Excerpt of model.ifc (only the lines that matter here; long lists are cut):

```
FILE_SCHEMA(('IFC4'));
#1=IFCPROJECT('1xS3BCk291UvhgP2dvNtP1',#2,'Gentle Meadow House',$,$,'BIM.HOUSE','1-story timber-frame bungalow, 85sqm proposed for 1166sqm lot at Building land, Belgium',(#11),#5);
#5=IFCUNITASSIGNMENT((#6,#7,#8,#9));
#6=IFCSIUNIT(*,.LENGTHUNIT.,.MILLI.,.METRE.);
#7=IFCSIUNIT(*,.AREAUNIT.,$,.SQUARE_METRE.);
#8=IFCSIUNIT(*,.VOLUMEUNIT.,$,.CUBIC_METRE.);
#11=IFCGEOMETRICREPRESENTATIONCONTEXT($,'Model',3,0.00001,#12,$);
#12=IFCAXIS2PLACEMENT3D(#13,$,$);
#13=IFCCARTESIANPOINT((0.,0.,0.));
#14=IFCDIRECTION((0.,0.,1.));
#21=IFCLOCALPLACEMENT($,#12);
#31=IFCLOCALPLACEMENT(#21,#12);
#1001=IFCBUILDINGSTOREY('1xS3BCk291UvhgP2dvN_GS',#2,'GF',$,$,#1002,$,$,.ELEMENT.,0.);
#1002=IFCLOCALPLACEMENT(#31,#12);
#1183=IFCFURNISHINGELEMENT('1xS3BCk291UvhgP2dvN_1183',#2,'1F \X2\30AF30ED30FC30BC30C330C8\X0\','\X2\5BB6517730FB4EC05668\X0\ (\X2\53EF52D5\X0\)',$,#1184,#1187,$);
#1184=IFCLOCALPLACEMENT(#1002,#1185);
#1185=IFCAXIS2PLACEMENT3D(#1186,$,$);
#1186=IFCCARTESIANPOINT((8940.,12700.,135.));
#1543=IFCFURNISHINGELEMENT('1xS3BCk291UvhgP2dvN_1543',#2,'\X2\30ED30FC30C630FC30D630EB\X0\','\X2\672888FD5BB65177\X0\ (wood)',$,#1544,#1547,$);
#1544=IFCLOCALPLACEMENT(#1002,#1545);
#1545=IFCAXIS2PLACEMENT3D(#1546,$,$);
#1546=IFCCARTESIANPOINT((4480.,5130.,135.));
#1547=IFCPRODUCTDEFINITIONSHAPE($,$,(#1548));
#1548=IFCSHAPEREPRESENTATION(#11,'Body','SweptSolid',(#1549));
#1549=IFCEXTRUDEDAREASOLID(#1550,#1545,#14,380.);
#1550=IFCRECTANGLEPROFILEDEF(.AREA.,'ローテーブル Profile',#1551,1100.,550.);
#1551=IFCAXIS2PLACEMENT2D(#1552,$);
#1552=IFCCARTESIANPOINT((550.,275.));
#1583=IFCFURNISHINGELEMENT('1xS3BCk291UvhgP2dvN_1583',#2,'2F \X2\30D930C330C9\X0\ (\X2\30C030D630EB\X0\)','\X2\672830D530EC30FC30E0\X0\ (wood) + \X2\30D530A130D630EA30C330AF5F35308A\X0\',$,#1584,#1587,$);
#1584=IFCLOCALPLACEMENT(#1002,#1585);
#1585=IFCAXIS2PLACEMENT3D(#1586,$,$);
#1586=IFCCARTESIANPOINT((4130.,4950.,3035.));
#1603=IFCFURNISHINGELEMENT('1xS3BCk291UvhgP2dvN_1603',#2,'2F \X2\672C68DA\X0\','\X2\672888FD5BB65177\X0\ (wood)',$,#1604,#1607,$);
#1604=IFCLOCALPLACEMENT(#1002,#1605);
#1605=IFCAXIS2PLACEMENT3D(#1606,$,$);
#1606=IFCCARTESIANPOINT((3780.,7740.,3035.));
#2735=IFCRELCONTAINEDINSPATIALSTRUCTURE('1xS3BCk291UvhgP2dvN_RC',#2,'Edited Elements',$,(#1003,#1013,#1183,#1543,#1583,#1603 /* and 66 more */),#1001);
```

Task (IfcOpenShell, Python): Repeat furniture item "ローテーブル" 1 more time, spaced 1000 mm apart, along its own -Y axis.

```python
import ifcopenshell
import ifcopenshell.api.geometry
import ifcopenshell.api.root
import ifcopenshell.util.element
import ifcopenshell.util.placement

model = ifcopenshell.open("model.ifc")


def reuse_history(source, copy):
    """copy_class also copies each property set's owner history, people and application; keep the originals."""
    for rel in copy.IsDefinedBy:
        if rel.is_a("IfcRelDefinesByProperties") and (history := rel.RelatingPropertyDefinition.OwnerHistory):
            rel.RelatingPropertyDefinition.OwnerHistory = source.OwnerHistory
            ifcopenshell.util.element.remove_deep2(model, history)


source = model.by_guid("1xS3BCk291UvhgP2dvN_1543")
base = ifcopenshell.util.placement.get_local_placement(source.ObjectPlacement)
step = -base[:3, 1] * 1000.0

for i in range(1, 2):
    copy = ifcopenshell.api.root.copy_class(model, product=source)
    copy.Representation = ifcopenshell.util.element.copy_deep(
        model, source.Representation, exclude=["IfcGeometricRepresentationContext", "IfcRepresentationMap"]
    )
    reuse_history(source, copy)
    matrix = base.copy()
    matrix[:3, 3] += i * step
    print("added at", matrix[:3, 3].round(3) + 0.0)
    ifcopenshell.api.geometry.edit_object_placement(model, product=copy, matrix=matrix, is_si=False)

model.write("model_rev.ifc")
```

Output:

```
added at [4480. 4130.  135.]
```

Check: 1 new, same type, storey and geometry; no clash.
